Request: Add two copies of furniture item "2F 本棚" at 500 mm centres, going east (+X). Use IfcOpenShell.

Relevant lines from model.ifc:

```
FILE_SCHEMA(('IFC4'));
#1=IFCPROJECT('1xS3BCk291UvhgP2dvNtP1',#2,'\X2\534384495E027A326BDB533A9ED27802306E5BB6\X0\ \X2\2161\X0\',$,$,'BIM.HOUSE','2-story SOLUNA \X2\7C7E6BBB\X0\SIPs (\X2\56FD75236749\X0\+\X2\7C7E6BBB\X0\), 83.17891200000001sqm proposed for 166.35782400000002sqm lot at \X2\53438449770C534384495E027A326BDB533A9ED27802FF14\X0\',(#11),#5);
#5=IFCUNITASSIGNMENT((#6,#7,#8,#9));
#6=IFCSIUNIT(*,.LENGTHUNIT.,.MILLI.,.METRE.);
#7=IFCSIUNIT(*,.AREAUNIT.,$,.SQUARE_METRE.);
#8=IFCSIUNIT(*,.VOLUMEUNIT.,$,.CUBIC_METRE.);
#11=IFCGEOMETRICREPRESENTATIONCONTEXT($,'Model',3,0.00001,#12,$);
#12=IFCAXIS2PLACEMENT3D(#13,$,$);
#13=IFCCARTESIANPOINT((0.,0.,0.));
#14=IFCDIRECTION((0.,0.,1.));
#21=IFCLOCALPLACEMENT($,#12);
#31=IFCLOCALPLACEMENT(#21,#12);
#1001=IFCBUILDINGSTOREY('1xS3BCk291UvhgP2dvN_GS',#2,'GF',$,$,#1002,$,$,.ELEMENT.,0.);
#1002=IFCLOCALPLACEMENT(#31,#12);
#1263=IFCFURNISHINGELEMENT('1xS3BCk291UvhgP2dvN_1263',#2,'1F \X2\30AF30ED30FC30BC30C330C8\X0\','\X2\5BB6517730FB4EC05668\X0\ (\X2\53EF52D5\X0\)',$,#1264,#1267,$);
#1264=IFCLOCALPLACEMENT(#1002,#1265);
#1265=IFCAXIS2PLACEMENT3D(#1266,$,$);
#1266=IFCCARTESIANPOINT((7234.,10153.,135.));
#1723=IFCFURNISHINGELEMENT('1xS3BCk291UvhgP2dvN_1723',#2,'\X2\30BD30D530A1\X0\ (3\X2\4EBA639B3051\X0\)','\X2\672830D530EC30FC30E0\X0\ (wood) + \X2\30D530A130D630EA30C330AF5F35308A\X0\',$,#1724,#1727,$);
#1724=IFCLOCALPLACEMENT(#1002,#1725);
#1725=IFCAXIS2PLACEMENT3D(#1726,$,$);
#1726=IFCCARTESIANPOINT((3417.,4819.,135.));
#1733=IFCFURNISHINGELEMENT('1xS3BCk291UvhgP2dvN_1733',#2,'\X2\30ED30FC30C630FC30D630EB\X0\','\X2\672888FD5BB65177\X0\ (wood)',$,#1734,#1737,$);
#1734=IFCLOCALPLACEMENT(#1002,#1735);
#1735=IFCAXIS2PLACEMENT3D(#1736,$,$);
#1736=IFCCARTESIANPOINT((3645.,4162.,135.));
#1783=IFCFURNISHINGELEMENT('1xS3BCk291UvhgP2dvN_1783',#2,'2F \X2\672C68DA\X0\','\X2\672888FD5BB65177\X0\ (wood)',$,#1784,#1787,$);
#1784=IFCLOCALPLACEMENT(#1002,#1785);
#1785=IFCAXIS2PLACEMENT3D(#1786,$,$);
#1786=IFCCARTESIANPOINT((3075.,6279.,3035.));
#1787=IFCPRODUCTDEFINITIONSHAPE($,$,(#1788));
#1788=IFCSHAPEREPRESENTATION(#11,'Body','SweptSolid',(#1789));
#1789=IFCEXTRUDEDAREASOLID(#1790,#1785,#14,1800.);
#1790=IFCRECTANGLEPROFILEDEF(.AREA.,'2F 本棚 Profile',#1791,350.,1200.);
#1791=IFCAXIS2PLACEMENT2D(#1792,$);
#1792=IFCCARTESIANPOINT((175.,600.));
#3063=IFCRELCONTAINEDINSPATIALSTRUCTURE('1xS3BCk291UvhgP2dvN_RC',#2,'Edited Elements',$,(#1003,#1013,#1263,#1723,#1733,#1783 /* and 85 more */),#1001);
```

```python
import numpy as np
import ifcopenshell
import ifcopenshell.api.geometry
import ifcopenshell.api.root
import ifcopenshell.util.element
import ifcopenshell.util.placement

model = ifcopenshell.open("model.ifc")


def reuse_history(source, copy):
    """copy_class also copies each property set's owner history, people and application; keep the originals."""
    for rel in copy.IsDefinedBy:
        if rel.is_a("IfcRelDefinesByProperties") and (history := rel.RelatingPropertyDefinition.OwnerHistory):
            rel.RelatingPropertyDefinition.OwnerHistory = source.OwnerHistory
            ifcopenshell.util.element.remove_deep2(model, history)


source = model.by_id(1783)
base = ifcopenshell.util.placement.get_local_placement(source.ObjectPlacement)
step = np.array([1.0, 0.0, 0.0]) * 500.0

for i in range(1, 3):
    copy = ifcopenshell.api.root.copy_class(model, product=source)
    copy.Representation = ifcopenshell.util.element.copy_deep(
        model, source.Representation, exclude=["IfcGeometricRepresentationContext", "IfcRepresentationMap"]
    )
    reuse_history(source, copy)
    matrix = base.copy()
    matrix[:3, 3] += i * step
    print("added at", matrix[:3, 3].round(3) + 0.0)
    ifcopenshell.api.geometry.edit_object_placement(model, product=copy, matrix=matrix, is_si=False)

model.write("model_v2.ifc")
```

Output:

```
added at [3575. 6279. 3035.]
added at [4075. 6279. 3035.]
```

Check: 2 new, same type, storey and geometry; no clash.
